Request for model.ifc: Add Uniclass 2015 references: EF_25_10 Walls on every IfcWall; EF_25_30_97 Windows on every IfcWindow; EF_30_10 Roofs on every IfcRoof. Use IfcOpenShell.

First a look at what the model holds.

```python
import ifcopenshell

model = ifcopenshell.open("model.ifc")
print(model.schema)
print("classifications:", [c.Name for c in model.by_type("IfcClassification")])
for ifc_class in ("IfcDoor", "IfcRoof", "IfcStair", "IfcWall", "IfcWindow"):
    print(ifc_class, len(model.by_type(ifc_class)))
```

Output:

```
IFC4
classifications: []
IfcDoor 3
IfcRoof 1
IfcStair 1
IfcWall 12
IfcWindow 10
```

```python
import ifcopenshell
import ifcopenshell.api.classification

model = ifcopenshell.open("model.ifc")

system = ifcopenshell.api.classification.add_classification(model, classification="Uniclass 2015")

codes = {
    "IfcWall": ("EF_25_10", "Walls"),
    "IfcWindow": ("EF_25_30_97", "Windows"),
    "IfcRoof": ("EF_30_10", "Roofs"),
}
for ifc_class, (code, name) in codes.items():
    products = model.by_type(ifc_class)
    ifcopenshell.api.classification.add_reference(
        model, products=products, classification=system, identification=code, name=name
    )
    print(code, len(products))

model.write("model_rev.ifc")
```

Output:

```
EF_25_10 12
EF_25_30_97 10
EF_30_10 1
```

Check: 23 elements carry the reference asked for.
